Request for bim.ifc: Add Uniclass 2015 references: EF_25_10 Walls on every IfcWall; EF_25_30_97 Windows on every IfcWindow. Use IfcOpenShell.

First a look at what the model holds.

```python
import ifcopenshell

model = ifcopenshell.open("bim.ifc")
print(model.schema)
print("classifications:", [c.Name for c in model.by_type("IfcClassification")])
for ifc_class in ("IfcDoor", "IfcRoof", "IfcStair", "IfcWall", "IfcWindow"):
    print(ifc_class, len(model.by_type(ifc_class)))
```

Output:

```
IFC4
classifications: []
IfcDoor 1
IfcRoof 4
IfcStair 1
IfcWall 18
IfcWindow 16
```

```python
import ifcopenshell
import ifcopenshell.api.classification

model = ifcopenshell.open("bim.ifc")

system = ifcopenshell.api.classification.add_classification(model, classification="Uniclass 2015")

codes = {
    "IfcWall": ("EF_25_10", "Walls"),
    "IfcWindow": ("EF_25_30_97", "Windows"),
}
for ifc_class, (code, name) in codes.items():
    products = model.by_type(ifc_class)
    ifcopenshell.api.classification.add_reference(
        model, products=products, classification=system, identification=code, name=name
    )
    print(code, len(products))

model.write("bim-out.ifc")
```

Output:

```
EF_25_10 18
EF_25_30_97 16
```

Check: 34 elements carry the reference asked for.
